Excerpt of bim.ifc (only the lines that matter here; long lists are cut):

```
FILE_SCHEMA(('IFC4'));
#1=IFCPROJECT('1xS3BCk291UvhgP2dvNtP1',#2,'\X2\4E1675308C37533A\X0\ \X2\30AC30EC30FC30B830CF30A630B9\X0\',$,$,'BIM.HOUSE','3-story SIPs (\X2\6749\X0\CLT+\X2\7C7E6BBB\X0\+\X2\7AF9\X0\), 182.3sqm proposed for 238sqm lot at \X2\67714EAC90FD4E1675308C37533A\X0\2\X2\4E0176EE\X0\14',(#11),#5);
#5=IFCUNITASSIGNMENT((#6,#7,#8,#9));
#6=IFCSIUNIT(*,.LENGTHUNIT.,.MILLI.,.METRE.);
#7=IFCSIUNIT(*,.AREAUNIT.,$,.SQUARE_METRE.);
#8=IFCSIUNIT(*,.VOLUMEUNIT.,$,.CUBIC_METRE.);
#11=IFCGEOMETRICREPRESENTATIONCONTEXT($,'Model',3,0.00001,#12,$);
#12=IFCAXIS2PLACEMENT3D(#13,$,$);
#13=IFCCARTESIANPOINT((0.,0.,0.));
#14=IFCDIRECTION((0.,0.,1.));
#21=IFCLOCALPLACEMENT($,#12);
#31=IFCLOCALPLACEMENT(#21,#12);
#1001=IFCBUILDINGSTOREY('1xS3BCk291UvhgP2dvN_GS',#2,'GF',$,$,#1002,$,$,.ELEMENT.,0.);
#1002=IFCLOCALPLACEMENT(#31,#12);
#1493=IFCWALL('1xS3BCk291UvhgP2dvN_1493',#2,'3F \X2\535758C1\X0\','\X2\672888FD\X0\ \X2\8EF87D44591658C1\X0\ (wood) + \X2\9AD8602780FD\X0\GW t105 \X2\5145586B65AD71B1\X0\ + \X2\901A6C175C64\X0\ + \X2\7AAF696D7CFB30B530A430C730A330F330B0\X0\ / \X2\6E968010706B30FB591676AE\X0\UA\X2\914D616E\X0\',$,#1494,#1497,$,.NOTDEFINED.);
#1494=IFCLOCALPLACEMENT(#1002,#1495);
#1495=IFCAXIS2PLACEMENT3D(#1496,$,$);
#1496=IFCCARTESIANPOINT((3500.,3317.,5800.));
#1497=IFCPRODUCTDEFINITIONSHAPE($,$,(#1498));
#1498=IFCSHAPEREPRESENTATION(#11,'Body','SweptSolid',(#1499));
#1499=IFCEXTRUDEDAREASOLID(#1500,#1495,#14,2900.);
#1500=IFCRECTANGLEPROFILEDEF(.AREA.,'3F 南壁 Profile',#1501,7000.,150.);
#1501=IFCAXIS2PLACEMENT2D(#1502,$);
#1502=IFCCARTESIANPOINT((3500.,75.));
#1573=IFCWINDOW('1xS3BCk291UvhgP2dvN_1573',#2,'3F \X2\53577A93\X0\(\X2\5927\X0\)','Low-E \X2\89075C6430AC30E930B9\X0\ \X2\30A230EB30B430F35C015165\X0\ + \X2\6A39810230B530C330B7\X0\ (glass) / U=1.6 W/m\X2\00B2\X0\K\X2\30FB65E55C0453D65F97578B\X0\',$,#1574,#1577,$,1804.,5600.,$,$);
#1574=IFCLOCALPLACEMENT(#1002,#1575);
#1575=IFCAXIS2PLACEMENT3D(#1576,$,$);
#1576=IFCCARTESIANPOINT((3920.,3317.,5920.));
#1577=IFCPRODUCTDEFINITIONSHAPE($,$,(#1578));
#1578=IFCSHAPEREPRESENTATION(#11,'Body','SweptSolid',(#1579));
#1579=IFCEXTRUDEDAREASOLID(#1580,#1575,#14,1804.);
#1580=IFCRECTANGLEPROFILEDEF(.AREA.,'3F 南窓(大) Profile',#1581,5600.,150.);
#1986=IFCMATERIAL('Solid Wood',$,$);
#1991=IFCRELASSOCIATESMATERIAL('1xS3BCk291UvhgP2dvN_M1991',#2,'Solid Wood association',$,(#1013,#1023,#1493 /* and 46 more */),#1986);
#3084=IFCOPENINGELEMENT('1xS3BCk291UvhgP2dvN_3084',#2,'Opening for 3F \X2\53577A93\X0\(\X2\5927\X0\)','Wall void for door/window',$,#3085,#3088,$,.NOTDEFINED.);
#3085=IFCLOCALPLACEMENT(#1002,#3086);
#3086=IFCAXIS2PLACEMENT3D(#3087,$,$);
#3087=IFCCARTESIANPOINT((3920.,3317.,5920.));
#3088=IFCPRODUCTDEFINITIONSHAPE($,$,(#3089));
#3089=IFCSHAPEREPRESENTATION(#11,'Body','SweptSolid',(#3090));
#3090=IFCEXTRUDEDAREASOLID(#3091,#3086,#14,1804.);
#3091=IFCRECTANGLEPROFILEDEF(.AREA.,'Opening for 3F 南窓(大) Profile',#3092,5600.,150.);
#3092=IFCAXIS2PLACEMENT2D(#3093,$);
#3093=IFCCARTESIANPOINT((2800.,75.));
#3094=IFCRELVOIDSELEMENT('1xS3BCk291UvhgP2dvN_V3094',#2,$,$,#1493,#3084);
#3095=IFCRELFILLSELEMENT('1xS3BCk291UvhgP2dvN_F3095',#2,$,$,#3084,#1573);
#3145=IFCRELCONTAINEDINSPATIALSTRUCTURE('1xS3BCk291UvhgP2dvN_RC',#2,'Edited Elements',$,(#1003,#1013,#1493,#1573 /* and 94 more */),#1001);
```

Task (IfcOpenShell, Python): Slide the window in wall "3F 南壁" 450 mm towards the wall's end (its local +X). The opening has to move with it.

```python
import ifcopenshell
import ifcopenshell.api.geometry
import ifcopenshell.util.placement

model = ifcopenshell.open("bim.ifc")

window = model.by_guid("1xS3BCk291UvhgP2dvN_1573")
opening = window.FillsVoids[0].RelatingOpeningElement
wall = opening.VoidsElements[0].RelatingBuildingElement

wall_matrix = ifcopenshell.util.placement.get_local_placement(wall.ObjectPlacement)
shift = wall_matrix[:3, 0] * 450.0
before = ifcopenshell.util.placement.get_local_placement(window.ObjectPlacement)[:3, 3].copy()

# The window is not placed relative to its opening, so move both.
for product in (opening, window):
    matrix = ifcopenshell.util.placement.get_local_placement(product.ObjectPlacement)
    matrix[:3, 3] += shift
    ifcopenshell.api.geometry.edit_object_placement(model, product=product, matrix=matrix, is_si=False)

after = ifcopenshell.util.placement.get_local_placement(window.ObjectPlacement)[:3, 3]
print("window moved by", (after - before).round(3) + 0.0)

model.write("bim_edited.ifc")
```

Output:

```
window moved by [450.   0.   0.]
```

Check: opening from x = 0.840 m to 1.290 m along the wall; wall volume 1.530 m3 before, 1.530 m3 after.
